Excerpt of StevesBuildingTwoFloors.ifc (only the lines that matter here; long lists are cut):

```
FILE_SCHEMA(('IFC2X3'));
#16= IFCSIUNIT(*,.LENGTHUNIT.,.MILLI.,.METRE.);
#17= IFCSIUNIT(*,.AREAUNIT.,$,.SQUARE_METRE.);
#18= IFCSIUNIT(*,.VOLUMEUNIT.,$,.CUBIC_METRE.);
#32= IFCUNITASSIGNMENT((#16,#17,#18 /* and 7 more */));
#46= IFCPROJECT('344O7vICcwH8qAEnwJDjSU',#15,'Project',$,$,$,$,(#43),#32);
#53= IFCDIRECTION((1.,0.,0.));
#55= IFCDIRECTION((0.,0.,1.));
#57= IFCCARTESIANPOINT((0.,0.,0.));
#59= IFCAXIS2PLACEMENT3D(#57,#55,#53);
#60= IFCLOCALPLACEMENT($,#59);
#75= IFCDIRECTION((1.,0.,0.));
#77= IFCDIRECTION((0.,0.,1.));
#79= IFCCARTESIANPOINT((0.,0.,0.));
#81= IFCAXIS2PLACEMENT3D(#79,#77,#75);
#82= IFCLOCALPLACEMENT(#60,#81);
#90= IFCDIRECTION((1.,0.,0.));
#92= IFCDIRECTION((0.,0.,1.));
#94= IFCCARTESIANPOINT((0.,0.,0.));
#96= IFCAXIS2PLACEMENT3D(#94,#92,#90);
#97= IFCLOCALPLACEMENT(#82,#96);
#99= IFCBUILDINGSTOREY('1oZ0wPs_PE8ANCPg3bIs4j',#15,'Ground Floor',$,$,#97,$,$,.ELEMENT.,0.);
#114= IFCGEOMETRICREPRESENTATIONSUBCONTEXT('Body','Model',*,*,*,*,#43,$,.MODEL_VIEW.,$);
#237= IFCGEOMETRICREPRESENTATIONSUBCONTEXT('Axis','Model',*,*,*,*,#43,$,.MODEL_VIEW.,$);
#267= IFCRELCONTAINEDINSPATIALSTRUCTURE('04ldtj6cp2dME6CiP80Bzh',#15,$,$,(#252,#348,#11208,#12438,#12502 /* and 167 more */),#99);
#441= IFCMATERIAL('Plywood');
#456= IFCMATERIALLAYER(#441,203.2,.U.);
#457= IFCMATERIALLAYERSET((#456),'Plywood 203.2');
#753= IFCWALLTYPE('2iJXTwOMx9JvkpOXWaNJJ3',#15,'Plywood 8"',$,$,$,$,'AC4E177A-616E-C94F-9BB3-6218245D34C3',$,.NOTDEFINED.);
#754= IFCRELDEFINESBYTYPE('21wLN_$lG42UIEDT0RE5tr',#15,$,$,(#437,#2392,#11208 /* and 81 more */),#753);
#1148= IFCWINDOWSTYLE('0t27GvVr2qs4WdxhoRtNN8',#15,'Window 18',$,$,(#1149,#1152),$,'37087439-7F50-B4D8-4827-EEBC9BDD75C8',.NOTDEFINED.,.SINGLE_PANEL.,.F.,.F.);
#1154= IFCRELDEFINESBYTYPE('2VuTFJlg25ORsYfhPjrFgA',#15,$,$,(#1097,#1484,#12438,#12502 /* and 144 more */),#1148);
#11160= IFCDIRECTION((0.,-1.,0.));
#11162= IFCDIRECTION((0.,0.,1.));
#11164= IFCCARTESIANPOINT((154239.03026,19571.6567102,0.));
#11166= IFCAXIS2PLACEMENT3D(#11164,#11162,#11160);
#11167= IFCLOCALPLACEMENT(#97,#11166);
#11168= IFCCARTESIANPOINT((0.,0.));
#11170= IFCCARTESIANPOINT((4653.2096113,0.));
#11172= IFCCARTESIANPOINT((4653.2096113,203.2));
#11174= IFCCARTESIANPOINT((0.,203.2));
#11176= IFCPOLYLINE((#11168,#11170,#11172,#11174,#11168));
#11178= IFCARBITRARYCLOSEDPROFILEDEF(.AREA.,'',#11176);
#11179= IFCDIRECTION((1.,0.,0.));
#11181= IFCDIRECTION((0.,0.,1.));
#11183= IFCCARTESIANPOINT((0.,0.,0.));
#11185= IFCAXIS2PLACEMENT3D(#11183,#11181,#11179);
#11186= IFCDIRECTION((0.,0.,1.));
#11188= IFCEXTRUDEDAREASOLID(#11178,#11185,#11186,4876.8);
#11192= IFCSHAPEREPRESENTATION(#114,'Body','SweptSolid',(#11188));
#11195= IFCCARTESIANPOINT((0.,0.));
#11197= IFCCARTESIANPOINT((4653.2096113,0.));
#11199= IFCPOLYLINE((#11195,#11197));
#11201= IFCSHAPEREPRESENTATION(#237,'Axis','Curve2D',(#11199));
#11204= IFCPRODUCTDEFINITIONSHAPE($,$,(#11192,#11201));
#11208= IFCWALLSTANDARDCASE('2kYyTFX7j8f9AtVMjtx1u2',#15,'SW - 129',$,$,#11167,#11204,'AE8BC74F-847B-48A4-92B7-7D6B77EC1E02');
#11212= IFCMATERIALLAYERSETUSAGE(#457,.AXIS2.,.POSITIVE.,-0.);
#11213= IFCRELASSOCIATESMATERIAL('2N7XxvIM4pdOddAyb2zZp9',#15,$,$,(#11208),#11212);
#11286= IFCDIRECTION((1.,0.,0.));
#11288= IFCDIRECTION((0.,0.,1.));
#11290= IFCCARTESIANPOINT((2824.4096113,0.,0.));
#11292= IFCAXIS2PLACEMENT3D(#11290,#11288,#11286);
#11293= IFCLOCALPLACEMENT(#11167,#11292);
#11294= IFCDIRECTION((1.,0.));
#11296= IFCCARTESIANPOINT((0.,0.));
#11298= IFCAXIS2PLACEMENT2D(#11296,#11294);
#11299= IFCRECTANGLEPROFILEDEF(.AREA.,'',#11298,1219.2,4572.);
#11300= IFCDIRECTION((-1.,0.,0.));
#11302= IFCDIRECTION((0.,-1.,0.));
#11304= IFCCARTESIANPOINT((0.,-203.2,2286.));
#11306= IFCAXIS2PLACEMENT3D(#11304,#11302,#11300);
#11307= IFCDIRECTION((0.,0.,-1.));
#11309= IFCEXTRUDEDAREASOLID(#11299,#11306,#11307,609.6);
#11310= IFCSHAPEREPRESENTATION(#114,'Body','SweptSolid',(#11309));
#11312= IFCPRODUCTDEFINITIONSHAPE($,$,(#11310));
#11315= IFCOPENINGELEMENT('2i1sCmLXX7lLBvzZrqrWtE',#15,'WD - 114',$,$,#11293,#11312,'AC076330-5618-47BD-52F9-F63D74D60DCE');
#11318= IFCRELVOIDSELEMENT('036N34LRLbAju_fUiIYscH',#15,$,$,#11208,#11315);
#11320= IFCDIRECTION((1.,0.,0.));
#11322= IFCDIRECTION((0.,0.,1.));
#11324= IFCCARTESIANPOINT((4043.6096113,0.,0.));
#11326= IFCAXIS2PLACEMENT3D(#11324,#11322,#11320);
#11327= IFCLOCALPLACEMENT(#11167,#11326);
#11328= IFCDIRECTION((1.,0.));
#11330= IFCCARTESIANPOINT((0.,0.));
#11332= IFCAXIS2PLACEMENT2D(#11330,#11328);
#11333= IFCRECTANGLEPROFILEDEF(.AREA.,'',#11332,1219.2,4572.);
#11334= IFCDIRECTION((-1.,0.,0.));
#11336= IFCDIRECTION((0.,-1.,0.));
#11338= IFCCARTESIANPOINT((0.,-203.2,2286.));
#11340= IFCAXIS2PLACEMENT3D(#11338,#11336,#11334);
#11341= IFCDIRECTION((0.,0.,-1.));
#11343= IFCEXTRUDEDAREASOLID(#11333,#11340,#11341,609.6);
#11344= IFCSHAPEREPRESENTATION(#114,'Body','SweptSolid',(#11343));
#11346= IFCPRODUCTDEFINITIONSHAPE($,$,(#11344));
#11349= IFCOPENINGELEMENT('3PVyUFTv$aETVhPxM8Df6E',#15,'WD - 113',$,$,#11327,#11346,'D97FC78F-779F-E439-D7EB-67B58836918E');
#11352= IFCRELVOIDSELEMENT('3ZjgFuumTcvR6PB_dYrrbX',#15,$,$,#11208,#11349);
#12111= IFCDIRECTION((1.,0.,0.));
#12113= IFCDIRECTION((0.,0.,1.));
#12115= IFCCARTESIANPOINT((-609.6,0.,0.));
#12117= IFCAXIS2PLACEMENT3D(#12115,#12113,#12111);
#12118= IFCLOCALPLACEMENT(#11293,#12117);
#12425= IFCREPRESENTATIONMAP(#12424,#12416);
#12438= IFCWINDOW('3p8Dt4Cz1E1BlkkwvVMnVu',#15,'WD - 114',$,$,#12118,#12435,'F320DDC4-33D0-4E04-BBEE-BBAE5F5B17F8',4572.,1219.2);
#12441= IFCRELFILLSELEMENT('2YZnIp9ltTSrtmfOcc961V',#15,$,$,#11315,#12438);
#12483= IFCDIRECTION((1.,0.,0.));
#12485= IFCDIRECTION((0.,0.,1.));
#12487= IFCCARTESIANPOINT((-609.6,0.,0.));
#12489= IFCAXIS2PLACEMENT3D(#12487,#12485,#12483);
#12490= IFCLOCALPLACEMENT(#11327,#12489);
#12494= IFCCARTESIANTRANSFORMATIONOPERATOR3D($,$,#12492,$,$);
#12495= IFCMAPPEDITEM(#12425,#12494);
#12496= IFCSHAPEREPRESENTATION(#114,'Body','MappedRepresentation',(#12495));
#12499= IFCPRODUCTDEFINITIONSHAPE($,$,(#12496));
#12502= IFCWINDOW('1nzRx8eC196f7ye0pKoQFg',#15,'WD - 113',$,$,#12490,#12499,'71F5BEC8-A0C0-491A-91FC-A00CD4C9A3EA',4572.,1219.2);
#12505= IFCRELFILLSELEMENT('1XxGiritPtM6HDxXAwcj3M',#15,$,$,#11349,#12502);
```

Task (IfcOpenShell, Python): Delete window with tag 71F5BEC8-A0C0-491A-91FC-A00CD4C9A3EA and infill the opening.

```python
import ifcopenshell
import ifcopenshell.api.feature
import ifcopenshell.api.root
import ifcopenshell.geom
import ifcopenshell.util.shape

model = ifcopenshell.open("StevesBuildingTwoFloors.ifc")
settings = ifcopenshell.geom.settings()


def volume(element):
    """Net volume in cubic metres, openings subtracted."""
    shape = ifcopenshell.geom.create_shape(settings, element)
    return ifcopenshell.util.shape.get_volume(shape.geometry)


window = model.by_id(12502)
opening = window.FillsVoids[0].RelatingOpeningElement
wall = opening.VoidsElements[0].RelatingBuildingElement
before = volume(wall)

ifcopenshell.api.root.remove_product(model, product=window)
ifcopenshell.api.feature.remove_feature(model, feature=opening)

after = volume(wall)

print(f"wall volume {before:.3f} -> {after:.3f} m3")

model.write("StevesBuildingTwoFloors_edited.ifc")
```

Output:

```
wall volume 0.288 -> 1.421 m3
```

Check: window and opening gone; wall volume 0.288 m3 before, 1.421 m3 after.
